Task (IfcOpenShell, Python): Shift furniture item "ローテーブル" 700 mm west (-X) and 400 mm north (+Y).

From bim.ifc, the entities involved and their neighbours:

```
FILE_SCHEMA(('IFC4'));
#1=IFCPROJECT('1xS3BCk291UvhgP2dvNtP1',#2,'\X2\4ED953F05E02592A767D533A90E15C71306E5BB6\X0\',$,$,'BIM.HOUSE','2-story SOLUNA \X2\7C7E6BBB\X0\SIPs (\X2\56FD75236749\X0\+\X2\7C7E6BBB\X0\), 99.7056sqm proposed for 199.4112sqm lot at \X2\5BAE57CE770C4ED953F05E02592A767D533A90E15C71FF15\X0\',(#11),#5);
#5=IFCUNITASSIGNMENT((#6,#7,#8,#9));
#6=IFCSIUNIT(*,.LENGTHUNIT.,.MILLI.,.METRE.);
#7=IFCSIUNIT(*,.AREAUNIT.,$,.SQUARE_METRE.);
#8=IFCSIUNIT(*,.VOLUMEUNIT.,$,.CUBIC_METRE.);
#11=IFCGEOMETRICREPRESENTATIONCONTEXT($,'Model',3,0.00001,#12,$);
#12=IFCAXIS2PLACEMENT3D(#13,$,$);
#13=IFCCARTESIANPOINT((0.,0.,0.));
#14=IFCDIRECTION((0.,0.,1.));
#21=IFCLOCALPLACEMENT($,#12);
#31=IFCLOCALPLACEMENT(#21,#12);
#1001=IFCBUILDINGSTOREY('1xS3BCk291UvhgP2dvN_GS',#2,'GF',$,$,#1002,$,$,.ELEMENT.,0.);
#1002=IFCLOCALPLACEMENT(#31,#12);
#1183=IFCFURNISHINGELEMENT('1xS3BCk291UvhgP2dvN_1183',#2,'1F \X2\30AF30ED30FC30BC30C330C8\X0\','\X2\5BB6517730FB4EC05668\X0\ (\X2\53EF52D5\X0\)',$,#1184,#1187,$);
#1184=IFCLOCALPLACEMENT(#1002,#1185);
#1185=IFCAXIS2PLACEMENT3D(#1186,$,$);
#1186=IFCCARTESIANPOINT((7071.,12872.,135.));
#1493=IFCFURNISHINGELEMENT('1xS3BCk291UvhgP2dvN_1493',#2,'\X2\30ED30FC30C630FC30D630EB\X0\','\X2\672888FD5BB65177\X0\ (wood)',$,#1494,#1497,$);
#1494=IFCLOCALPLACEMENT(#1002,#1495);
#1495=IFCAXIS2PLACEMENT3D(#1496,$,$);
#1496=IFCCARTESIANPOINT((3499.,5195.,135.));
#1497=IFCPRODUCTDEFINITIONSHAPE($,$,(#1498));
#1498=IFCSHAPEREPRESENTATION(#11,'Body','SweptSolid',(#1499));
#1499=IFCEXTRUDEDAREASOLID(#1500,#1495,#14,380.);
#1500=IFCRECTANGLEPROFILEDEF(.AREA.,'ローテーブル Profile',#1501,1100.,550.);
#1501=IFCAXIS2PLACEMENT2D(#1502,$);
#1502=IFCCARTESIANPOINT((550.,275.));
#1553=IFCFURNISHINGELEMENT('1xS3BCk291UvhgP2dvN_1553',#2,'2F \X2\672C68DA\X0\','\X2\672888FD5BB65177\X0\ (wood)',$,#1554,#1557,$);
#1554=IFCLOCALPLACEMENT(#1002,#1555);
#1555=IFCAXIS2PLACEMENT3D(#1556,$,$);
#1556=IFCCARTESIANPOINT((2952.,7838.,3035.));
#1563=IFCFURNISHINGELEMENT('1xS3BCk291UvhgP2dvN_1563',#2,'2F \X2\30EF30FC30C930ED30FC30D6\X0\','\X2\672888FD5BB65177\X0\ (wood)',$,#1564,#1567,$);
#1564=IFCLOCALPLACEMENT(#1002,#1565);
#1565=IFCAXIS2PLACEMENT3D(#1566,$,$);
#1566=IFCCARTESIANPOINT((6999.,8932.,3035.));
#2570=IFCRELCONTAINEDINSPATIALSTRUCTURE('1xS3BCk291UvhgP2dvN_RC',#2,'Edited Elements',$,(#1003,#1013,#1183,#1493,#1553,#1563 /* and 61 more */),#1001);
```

```python
import ifcopenshell
import ifcopenshell.api.geometry
import ifcopenshell.util.placement
import ifcopenshell.util.unit

model = ifcopenshell.open("bim.ifc")
unit_scale = ifcopenshell.util.unit.calculate_unit_scale(model)

item = model.by_guid("1xS3BCk291UvhgP2dvN_1493")
matrix = ifcopenshell.util.placement.get_local_placement(item.ObjectPlacement)
matrix[0, 3] -= 0.7 / unit_scale
matrix[1, 3] += 0.4 / unit_scale
ifcopenshell.api.geometry.edit_object_placement(model, product=item, matrix=matrix, is_si=False)

print(ifcopenshell.util.placement.get_local_placement(item.ObjectPlacement).round(3) + 0.0)

model.write("bim_v2.ifc")
```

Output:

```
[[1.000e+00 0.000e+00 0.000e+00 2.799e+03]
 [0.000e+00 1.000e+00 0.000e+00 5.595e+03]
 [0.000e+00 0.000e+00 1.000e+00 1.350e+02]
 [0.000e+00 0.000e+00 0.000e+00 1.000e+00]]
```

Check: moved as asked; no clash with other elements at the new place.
